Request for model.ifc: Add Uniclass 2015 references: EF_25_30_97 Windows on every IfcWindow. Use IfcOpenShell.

First a look at what the model holds.

```python
import ifcopenshell

model = ifcopenshell.open("model.ifc")
print(model.schema)
print("classifications:", [c.Name for c in model.by_type("IfcClassification")])
for ifc_class in ("IfcDoor", "IfcRoof", "IfcStair", "IfcWall", "IfcWindow"):
    print(ifc_class, len(model.by_type(ifc_class)))
```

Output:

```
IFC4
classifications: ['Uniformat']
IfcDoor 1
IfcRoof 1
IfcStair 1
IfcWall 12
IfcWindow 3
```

```python
import ifcopenshell
import ifcopenshell.api.classification

model = ifcopenshell.open("model.ifc")

system = ifcopenshell.api.classification.add_classification(model, classification="Uniclass 2015")

codes = {
    "IfcWindow": ("EF_25_30_97", "Windows"),
}
for ifc_class, (code, name) in codes.items():
    products = model.by_type(ifc_class)
    ifcopenshell.api.classification.add_reference(
        model, products=products, classification=system, identification=code, name=name
    )
    print(code, len(products))

model.write("model_edited.ifc")
```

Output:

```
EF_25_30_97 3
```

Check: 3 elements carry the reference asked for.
